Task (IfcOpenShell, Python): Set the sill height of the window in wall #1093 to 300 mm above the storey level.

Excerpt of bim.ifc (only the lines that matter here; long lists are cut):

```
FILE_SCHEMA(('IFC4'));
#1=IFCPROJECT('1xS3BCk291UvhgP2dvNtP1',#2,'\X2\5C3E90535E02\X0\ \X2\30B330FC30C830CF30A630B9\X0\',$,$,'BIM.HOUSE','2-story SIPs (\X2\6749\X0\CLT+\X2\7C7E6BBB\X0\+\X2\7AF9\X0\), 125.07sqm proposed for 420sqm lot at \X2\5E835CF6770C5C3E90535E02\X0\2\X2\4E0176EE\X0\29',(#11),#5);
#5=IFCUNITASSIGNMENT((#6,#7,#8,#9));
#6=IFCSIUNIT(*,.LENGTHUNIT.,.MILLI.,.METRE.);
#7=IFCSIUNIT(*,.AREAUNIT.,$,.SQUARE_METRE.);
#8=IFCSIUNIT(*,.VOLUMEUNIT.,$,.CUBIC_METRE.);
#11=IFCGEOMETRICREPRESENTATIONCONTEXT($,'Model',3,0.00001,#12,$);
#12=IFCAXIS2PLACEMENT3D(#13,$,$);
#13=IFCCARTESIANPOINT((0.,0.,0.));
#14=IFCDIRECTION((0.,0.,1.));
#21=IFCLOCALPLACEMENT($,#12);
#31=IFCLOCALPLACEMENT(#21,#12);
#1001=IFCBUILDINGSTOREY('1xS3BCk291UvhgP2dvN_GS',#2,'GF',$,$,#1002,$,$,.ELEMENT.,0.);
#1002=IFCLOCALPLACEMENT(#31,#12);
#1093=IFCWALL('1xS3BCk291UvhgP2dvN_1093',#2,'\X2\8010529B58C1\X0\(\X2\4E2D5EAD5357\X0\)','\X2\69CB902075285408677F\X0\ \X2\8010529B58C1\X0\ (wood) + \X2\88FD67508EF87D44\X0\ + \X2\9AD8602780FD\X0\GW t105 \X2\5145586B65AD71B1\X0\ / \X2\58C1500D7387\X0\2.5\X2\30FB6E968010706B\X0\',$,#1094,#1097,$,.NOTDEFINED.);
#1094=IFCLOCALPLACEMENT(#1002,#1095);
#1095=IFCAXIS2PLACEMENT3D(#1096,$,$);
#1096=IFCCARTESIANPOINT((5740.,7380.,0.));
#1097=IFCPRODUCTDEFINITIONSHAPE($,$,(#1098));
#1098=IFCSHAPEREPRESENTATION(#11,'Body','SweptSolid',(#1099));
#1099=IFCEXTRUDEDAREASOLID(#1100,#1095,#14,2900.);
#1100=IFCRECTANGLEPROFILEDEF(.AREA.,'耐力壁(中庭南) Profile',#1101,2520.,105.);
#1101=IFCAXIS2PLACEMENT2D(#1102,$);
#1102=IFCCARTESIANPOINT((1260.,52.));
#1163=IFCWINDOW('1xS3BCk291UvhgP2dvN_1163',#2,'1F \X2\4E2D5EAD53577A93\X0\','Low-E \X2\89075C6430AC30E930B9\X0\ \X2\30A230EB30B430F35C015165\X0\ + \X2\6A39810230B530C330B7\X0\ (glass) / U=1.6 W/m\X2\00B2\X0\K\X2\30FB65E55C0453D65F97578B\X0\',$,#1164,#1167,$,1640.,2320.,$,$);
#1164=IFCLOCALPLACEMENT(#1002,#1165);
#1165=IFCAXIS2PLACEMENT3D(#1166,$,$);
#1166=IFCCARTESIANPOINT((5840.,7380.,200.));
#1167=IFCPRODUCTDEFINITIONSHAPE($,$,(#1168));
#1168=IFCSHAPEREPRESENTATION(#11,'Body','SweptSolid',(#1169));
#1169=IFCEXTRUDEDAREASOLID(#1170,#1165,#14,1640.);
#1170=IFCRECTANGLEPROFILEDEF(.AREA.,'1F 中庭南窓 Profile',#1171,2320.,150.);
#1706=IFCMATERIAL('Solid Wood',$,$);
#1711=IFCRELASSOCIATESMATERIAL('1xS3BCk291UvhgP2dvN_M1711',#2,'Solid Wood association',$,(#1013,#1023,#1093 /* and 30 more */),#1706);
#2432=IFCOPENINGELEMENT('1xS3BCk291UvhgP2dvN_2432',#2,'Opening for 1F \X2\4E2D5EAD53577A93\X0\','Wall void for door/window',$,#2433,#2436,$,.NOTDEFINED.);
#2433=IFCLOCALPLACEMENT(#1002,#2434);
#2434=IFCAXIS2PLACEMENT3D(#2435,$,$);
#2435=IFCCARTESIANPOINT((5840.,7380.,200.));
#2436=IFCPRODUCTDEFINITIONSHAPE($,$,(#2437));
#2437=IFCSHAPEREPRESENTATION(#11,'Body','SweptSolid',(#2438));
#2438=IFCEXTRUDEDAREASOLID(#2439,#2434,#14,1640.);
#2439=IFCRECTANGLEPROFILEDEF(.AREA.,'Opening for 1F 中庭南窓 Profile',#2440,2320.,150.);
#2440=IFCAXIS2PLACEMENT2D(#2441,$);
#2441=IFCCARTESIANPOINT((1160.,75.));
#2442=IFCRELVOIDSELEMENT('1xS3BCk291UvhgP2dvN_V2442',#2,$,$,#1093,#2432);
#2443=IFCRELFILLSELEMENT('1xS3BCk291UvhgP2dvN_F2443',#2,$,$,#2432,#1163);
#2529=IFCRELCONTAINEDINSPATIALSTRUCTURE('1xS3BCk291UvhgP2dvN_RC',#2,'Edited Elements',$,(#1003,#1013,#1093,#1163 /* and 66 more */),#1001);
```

```python
import numpy as np
import ifcopenshell
import ifcopenshell.api.geometry
import ifcopenshell.geom
import ifcopenshell.util.element
import ifcopenshell.util.placement
import ifcopenshell.util.shape
import ifcopenshell.util.unit

model = ifcopenshell.open("bim.ifc")
unit_scale = ifcopenshell.util.unit.calculate_unit_scale(model)

window = model.by_guid("1xS3BCk291UvhgP2dvN_1163")
opening = window.FillsVoids[0].RelatingOpeningElement
storey = ifcopenshell.util.element.get_container(window, ifc_class="IfcBuildingStorey")
level = ifcopenshell.util.placement.get_local_placement(storey.ObjectPlacement)[2, 3]

# The opening's origin need not be at the sill, so measure its lowest point.
shape = ifcopenshell.geom.create_shape(ifcopenshell.geom.settings(), opening)
bottom = ifcopenshell.util.shape.get_shape_bottom_elevation(shape, shape.geometry) / unit_scale
dz = level + 0.3 / unit_scale - bottom

shift = np.array([0.0, 0.0, dz])
# The window is not placed relative to its opening, so move both.
for product in (opening, window):
    matrix = ifcopenshell.util.placement.get_local_placement(product.ObjectPlacement)
    matrix[:3, 3] += shift
    ifcopenshell.api.geometry.edit_object_placement(model, product=product, matrix=matrix, is_si=False)

print(f"moved by {dz * unit_scale:+.3f} m")

model.write("bim-out.ifc")
```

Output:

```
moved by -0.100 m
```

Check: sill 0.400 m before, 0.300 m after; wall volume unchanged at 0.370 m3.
